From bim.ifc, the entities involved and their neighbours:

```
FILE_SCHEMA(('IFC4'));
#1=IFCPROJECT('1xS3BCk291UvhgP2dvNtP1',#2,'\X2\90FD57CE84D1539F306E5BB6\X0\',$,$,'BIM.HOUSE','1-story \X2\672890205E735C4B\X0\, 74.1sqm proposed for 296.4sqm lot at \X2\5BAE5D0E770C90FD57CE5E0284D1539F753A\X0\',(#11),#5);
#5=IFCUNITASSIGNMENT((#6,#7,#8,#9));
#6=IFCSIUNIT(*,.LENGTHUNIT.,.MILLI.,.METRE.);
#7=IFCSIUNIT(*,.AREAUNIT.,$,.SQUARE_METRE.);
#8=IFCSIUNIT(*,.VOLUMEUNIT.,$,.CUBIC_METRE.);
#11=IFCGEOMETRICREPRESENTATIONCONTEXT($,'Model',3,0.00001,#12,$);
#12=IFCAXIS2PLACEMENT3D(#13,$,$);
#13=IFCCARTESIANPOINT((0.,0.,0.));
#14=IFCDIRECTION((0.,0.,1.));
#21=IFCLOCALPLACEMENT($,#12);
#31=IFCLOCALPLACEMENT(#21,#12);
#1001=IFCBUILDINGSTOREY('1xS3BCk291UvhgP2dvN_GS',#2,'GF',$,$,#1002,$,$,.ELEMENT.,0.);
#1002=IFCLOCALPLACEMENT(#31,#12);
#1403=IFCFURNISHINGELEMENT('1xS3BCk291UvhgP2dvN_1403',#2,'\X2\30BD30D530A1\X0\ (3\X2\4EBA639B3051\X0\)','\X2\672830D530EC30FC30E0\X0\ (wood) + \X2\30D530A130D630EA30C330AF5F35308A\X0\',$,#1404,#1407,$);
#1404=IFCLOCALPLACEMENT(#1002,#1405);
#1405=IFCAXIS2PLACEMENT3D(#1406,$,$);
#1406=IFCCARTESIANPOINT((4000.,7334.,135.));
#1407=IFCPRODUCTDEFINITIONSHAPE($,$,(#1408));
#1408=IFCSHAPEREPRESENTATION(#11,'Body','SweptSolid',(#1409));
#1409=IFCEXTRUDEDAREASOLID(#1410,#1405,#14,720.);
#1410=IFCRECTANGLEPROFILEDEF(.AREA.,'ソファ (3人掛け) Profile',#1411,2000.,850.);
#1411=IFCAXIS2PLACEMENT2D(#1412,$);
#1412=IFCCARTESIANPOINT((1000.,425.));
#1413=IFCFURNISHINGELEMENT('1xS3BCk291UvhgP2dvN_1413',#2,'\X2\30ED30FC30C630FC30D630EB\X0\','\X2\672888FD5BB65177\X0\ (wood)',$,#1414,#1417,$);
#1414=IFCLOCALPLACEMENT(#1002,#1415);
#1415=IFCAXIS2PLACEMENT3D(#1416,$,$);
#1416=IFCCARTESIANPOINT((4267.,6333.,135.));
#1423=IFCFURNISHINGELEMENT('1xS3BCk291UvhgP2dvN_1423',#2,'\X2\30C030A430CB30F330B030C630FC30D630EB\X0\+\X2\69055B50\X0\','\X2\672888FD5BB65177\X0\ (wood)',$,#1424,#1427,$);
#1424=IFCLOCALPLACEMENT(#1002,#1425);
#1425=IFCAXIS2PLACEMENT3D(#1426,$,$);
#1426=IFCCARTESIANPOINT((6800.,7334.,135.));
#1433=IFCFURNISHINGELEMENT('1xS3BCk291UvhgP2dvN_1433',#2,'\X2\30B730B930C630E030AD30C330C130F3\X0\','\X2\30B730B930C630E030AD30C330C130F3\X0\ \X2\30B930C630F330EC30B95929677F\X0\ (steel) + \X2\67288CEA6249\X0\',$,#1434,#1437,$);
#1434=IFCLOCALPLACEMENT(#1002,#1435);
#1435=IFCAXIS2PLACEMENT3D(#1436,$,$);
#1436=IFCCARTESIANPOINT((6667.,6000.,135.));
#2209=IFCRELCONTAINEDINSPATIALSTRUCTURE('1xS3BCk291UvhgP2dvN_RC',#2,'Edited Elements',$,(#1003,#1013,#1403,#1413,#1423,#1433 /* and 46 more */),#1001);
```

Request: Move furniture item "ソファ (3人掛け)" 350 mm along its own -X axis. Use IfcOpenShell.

```python
import ifcopenshell
import ifcopenshell.api.geometry
import ifcopenshell.util.placement
import ifcopenshell.util.unit

model = ifcopenshell.open("bim.ifc")
unit_scale = ifcopenshell.util.unit.calculate_unit_scale(model)

item = model.by_guid("1xS3BCk291UvhgP2dvN_1403")
matrix = ifcopenshell.util.placement.get_local_placement(item.ObjectPlacement)
matrix[:3, 3] -= matrix[:3, 0] * 0.35 / unit_scale
ifcopenshell.api.geometry.edit_object_placement(model, product=item, matrix=matrix, is_si=False)

print(ifcopenshell.util.placement.get_local_placement(item.ObjectPlacement).round(3) + 0.0)

model.write("bim_edited.ifc")
```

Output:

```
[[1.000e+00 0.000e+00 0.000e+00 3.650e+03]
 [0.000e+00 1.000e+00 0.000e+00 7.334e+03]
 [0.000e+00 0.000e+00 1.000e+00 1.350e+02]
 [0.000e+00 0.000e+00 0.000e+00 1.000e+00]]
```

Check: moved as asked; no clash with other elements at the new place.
